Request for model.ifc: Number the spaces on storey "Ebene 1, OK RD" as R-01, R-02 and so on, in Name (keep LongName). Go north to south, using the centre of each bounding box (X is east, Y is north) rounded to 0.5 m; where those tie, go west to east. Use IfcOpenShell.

First a look at what the model holds.

```python
import ifcopenshell
import ifcopenshell.util.element
import ifcopenshell.util.placement

model = ifcopenshell.open("model.ifc")
print(model.schema)
storey = next(s for s in model.by_type("IfcBuildingStorey") if s.Name == "Ebene 1, OK RD")
spaces = [e for e in ifcopenshell.util.element.get_decomposition(storey) if e.is_a("IfcSpace")]
for e in sorted(spaces, key=lambda e: e.id()):
    origin = ifcopenshell.util.placement.get_local_placement(e.ObjectPlacement)[:3, 3]
    print(e.id(), e.Name, e.LongName, origin.round(2) + 0.0, sep=" | ")
```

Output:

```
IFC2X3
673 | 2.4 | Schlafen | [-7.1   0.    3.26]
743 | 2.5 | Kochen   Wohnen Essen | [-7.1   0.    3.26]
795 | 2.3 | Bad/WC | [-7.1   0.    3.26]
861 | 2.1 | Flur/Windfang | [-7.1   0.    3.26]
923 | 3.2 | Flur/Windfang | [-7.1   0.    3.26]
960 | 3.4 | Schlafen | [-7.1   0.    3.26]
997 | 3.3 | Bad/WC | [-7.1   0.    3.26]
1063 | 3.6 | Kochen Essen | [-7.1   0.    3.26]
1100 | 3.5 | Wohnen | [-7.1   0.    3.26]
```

```python
import ifcopenshell
import ifcopenshell.geom
import ifcopenshell.util.element
import ifcopenshell.util.shape

model = ifcopenshell.open("model.ifc")
settings = ifcopenshell.geom.settings()
settings.set("use-world-coords", True)


def centre(element):
    shape = ifcopenshell.geom.create_shape(settings, element)
    return ifcopenshell.util.shape.get_bbox_centroid(shape.geometry)


storey = next(s for s in model.by_type("IfcBuildingStorey") if s.Name == "Ebene 1, OK RD")
spaces = [e for e in ifcopenshell.util.element.get_decomposition(storey) if e.is_a("IfcSpace")]

# Insertion points can sit at a corner or the storey origin, so sort by the geometry (in metres).
centres = {e: centre(e) for e in spaces}
spaces.sort(key=lambda e: (-round(centres[e][1] / 0.5), centres[e][0]))

for i, e in enumerate(spaces, start=1):
    number = f"R-{i:02d}"
    e.Name = number
    print(e.id(), number)

model.write("model-out.ifc")
```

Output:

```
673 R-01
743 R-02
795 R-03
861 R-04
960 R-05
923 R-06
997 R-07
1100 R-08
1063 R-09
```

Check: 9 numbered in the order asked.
